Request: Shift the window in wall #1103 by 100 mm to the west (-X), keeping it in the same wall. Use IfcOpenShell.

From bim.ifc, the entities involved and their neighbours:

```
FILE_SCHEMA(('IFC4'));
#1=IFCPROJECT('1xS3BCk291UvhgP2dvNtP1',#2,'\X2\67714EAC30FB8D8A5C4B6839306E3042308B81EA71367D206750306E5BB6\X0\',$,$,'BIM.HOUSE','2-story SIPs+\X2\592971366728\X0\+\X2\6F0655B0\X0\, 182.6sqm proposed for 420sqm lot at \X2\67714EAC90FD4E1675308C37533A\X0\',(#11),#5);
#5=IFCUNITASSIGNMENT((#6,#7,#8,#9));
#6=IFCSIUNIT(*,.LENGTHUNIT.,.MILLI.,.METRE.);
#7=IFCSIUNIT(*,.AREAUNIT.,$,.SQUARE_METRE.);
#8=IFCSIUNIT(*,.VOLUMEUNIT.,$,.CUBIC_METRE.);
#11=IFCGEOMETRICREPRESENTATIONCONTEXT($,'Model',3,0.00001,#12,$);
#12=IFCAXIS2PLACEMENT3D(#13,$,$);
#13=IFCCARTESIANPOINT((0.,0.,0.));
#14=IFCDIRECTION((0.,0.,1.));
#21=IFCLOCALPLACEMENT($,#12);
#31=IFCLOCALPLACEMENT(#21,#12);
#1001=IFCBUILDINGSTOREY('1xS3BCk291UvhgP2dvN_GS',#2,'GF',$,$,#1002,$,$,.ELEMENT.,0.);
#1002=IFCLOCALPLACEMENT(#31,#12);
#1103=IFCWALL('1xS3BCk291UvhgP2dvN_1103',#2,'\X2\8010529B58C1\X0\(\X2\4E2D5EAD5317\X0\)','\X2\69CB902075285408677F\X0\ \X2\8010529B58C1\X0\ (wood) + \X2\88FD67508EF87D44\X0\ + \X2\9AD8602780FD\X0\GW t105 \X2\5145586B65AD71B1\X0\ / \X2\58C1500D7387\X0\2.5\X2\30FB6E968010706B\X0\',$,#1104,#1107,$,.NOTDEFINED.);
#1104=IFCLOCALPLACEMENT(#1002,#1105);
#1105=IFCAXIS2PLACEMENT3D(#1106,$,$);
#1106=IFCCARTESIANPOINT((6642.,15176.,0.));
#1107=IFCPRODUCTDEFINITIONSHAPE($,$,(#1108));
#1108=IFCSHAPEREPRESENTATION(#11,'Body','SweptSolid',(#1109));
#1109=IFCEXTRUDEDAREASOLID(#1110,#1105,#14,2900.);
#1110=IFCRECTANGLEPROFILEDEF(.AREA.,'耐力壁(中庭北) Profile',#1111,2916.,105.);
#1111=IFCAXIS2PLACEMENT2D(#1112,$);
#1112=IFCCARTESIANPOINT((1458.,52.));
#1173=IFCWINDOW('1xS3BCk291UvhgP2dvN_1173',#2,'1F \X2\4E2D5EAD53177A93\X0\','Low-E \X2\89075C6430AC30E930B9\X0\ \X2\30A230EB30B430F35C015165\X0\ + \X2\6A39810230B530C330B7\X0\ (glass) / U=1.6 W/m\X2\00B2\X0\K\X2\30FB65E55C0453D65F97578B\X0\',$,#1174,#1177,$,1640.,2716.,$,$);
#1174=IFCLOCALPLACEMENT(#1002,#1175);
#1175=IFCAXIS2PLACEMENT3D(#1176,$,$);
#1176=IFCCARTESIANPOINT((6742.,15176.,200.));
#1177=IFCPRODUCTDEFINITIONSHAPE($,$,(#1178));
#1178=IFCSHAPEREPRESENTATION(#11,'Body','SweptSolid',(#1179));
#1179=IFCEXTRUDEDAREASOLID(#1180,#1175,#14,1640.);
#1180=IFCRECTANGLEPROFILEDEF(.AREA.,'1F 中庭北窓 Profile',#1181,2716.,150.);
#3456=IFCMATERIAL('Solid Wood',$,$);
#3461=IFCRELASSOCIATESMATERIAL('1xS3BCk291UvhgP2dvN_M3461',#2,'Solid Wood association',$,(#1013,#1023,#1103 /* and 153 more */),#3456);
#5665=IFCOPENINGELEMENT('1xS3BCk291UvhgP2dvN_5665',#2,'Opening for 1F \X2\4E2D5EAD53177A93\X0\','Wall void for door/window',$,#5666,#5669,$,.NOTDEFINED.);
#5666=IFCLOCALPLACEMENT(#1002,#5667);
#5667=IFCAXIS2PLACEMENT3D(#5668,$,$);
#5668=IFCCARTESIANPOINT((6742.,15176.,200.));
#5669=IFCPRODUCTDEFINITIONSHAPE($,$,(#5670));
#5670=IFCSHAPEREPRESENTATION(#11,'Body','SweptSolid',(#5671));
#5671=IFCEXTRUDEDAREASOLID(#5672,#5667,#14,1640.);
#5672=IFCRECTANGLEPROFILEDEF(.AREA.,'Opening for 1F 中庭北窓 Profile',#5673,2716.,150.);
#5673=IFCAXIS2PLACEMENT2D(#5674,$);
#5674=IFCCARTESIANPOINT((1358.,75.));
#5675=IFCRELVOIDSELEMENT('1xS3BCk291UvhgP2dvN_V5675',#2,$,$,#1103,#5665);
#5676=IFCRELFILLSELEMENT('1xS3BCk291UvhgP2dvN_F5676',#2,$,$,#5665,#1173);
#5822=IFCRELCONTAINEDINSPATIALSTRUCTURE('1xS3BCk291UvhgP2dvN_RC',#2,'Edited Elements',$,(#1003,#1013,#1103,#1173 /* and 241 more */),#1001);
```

```python
import ifcopenshell
import ifcopenshell.api.geometry
import ifcopenshell.util.placement
import ifcopenshell.util.unit

model = ifcopenshell.open("bim.ifc")
unit_scale = ifcopenshell.util.unit.calculate_unit_scale(model)

window = model.by_guid("1xS3BCk291UvhgP2dvN_1173")
opening = window.FillsVoids[0].RelatingOpeningElement
wall = opening.VoidsElements[0].RelatingBuildingElement

wall_matrix = ifcopenshell.util.placement.get_local_placement(wall.ObjectPlacement)
shift = wall_matrix[:3, 0] * -0.1 / unit_scale
before = ifcopenshell.util.placement.get_local_placement(window.ObjectPlacement)[:3, 3].copy()

# The window is not placed relative to its opening, so move both.
for product in (opening, window):
    matrix = ifcopenshell.util.placement.get_local_placement(product.ObjectPlacement)
    matrix[:3, 3] += shift
    ifcopenshell.api.geometry.edit_object_placement(model, product=product, matrix=matrix, is_si=False)

after = ifcopenshell.util.placement.get_local_placement(window.ObjectPlacement)[:3, 3]
print("window moved by", (after - before).round(3) + 0.0)

model.write("bim_updated.ifc")
```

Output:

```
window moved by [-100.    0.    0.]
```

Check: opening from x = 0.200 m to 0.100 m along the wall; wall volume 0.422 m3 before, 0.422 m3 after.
